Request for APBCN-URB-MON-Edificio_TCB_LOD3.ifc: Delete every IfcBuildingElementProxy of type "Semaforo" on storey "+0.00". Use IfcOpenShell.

First a look at what the model holds.

```python
import ifcopenshell
import ifcopenshell.util.element

model = ifcopenshell.open("APBCN-URB-MON-Edificio_TCB_LOD3.ifc")
print(model.schema)
storey = next(s for s in model.by_type("IfcBuildingStorey") if s.Name == "+0.00")
proxies = [e for e in ifcopenshell.util.element.get_decomposition(storey) if e.is_a("IfcBuildingElementProxy")]
seen = {}
for e in proxies:
    element_type = ifcopenshell.util.element.get_type(e)
    name = element_type.Name if element_type not in (None, e) else None
    seen[name] = seen.get(name, 0) + 1
for name, count in sorted(seen.items(), key=str):
    print(count, "x", name)
```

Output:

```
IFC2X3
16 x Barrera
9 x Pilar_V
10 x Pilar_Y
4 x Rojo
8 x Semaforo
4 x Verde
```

```python
import ifcopenshell
import ifcopenshell.api.root
import ifcopenshell.util.element

model = ifcopenshell.open("APBCN-URB-MON-Edificio_TCB_LOD3.ifc")

storey = next(s for s in model.by_type("IfcBuildingStorey") if s.Name == "+0.00")
proxies = [e for e in ifcopenshell.util.element.get_decomposition(storey) if e.is_a("IfcBuildingElementProxy")]
targets = [e for e in proxies if (t := ifcopenshell.util.element.get_type(e)) not in (None, e) and t.Name == "Semaforo"]

for e in targets:
    ifcopenshell.api.root.remove_product(model, product=e)
print(len(targets), "removed")

model.write("APBCN-URB-MON-Edificio_TCB_LOD3_updated.ifc")
```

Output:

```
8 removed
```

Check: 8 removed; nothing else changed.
